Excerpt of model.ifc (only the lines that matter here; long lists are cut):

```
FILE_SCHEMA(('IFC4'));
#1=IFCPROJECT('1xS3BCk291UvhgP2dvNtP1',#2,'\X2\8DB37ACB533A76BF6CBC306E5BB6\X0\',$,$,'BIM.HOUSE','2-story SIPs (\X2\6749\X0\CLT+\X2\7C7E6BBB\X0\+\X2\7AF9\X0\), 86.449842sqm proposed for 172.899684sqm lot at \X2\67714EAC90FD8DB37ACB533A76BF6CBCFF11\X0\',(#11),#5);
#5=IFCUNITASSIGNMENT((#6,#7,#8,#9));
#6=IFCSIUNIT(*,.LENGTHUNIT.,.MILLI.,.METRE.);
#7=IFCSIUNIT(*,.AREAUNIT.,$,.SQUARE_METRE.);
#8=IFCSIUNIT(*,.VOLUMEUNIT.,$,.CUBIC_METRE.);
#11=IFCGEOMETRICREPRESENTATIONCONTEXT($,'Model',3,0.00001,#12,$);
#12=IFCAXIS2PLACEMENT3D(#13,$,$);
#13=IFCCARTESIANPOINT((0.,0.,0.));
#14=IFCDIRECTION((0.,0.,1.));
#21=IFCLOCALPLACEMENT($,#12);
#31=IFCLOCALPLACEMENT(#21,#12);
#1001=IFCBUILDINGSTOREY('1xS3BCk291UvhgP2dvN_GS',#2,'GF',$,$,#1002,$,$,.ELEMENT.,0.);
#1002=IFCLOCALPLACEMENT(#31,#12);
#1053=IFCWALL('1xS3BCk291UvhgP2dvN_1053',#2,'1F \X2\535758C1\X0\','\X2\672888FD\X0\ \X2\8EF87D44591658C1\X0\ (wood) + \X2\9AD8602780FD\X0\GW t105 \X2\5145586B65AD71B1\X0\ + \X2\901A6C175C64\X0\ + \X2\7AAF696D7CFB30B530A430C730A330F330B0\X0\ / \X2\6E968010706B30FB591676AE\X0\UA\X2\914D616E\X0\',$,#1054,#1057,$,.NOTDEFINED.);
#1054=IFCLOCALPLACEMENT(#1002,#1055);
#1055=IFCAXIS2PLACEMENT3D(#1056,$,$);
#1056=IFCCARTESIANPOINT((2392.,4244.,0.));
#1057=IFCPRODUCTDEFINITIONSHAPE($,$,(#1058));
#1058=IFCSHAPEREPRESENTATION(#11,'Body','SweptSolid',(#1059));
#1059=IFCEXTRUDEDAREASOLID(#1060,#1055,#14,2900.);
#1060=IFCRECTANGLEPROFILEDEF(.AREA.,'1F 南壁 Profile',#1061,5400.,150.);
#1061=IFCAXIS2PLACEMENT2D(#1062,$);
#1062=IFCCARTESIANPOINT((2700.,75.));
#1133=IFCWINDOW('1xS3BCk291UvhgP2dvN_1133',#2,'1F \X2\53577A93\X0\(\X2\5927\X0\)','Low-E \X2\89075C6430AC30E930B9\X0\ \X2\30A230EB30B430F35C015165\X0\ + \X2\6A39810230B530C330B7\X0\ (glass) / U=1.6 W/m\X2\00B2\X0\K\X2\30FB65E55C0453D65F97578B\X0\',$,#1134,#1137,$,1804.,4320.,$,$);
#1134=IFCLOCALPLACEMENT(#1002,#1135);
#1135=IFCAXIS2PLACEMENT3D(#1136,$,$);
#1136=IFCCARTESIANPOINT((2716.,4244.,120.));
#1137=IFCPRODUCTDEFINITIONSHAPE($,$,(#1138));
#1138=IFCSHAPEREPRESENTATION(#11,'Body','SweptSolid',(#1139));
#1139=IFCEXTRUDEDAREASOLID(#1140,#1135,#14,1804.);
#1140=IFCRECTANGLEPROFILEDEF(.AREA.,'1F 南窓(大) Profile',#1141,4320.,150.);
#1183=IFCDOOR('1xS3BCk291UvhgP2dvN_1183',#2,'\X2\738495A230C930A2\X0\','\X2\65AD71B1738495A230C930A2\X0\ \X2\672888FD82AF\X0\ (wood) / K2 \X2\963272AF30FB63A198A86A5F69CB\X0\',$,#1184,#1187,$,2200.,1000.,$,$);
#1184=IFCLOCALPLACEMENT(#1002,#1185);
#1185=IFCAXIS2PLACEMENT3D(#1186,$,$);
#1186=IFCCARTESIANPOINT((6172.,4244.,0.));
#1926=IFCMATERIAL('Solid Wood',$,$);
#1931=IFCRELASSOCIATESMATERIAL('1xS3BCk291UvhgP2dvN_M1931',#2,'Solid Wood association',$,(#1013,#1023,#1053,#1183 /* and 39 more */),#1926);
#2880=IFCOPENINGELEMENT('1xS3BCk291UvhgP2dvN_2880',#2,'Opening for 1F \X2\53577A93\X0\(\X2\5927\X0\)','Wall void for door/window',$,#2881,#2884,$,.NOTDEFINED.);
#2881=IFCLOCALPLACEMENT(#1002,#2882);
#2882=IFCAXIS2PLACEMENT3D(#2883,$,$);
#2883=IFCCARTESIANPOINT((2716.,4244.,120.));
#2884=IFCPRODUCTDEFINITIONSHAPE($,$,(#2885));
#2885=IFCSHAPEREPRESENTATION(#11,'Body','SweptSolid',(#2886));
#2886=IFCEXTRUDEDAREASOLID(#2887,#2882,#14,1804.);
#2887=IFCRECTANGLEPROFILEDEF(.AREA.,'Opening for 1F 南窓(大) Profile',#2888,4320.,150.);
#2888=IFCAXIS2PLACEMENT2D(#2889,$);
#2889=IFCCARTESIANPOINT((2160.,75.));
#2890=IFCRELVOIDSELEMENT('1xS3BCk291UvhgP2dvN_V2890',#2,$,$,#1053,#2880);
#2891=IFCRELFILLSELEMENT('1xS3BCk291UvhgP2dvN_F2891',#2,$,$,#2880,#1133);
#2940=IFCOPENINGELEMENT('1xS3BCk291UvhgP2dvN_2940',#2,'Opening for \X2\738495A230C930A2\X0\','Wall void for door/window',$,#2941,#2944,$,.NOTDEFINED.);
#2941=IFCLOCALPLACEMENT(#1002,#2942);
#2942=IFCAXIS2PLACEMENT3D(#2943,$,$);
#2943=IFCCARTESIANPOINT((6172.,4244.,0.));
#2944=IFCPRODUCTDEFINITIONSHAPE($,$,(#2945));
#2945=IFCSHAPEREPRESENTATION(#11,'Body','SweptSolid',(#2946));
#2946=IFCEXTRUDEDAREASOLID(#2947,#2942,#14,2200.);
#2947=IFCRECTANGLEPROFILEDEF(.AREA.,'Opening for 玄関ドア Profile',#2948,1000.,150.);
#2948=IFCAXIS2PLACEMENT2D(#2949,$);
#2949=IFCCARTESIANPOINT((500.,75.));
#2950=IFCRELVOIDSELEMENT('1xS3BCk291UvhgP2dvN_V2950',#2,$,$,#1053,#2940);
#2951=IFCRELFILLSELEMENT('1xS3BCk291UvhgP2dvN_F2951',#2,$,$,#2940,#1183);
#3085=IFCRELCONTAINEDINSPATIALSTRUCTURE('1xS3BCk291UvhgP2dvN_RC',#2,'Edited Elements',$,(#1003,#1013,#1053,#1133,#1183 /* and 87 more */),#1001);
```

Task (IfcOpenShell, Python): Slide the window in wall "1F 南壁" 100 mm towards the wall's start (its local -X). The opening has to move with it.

```python
import ifcopenshell
import ifcopenshell.api.geometry
import ifcopenshell.util.placement

model = ifcopenshell.open("model.ifc")

window = model.by_guid("1xS3BCk291UvhgP2dvN_1133")
opening = window.FillsVoids[0].RelatingOpeningElement
wall = opening.VoidsElements[0].RelatingBuildingElement

wall_matrix = ifcopenshell.util.placement.get_local_placement(wall.ObjectPlacement)
shift = wall_matrix[:3, 0] * -100.0
before = ifcopenshell.util.placement.get_local_placement(window.ObjectPlacement)[:3, 3].copy()

# The window is not placed relative to its opening, so move both.
for product in (opening, window):
    matrix = ifcopenshell.util.placement.get_local_placement(product.ObjectPlacement)
    matrix[:3, 3] += shift
    ifcopenshell.api.geometry.edit_object_placement(model, product=product, matrix=matrix, is_si=False)

after = ifcopenshell.util.placement.get_local_placement(window.ObjectPlacement)[:3, 3]
print("window moved by", (after - before).round(3) + 0.0)

model.write("model_updated.ifc")
```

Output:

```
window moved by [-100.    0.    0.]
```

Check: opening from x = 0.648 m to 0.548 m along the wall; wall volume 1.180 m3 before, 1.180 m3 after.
